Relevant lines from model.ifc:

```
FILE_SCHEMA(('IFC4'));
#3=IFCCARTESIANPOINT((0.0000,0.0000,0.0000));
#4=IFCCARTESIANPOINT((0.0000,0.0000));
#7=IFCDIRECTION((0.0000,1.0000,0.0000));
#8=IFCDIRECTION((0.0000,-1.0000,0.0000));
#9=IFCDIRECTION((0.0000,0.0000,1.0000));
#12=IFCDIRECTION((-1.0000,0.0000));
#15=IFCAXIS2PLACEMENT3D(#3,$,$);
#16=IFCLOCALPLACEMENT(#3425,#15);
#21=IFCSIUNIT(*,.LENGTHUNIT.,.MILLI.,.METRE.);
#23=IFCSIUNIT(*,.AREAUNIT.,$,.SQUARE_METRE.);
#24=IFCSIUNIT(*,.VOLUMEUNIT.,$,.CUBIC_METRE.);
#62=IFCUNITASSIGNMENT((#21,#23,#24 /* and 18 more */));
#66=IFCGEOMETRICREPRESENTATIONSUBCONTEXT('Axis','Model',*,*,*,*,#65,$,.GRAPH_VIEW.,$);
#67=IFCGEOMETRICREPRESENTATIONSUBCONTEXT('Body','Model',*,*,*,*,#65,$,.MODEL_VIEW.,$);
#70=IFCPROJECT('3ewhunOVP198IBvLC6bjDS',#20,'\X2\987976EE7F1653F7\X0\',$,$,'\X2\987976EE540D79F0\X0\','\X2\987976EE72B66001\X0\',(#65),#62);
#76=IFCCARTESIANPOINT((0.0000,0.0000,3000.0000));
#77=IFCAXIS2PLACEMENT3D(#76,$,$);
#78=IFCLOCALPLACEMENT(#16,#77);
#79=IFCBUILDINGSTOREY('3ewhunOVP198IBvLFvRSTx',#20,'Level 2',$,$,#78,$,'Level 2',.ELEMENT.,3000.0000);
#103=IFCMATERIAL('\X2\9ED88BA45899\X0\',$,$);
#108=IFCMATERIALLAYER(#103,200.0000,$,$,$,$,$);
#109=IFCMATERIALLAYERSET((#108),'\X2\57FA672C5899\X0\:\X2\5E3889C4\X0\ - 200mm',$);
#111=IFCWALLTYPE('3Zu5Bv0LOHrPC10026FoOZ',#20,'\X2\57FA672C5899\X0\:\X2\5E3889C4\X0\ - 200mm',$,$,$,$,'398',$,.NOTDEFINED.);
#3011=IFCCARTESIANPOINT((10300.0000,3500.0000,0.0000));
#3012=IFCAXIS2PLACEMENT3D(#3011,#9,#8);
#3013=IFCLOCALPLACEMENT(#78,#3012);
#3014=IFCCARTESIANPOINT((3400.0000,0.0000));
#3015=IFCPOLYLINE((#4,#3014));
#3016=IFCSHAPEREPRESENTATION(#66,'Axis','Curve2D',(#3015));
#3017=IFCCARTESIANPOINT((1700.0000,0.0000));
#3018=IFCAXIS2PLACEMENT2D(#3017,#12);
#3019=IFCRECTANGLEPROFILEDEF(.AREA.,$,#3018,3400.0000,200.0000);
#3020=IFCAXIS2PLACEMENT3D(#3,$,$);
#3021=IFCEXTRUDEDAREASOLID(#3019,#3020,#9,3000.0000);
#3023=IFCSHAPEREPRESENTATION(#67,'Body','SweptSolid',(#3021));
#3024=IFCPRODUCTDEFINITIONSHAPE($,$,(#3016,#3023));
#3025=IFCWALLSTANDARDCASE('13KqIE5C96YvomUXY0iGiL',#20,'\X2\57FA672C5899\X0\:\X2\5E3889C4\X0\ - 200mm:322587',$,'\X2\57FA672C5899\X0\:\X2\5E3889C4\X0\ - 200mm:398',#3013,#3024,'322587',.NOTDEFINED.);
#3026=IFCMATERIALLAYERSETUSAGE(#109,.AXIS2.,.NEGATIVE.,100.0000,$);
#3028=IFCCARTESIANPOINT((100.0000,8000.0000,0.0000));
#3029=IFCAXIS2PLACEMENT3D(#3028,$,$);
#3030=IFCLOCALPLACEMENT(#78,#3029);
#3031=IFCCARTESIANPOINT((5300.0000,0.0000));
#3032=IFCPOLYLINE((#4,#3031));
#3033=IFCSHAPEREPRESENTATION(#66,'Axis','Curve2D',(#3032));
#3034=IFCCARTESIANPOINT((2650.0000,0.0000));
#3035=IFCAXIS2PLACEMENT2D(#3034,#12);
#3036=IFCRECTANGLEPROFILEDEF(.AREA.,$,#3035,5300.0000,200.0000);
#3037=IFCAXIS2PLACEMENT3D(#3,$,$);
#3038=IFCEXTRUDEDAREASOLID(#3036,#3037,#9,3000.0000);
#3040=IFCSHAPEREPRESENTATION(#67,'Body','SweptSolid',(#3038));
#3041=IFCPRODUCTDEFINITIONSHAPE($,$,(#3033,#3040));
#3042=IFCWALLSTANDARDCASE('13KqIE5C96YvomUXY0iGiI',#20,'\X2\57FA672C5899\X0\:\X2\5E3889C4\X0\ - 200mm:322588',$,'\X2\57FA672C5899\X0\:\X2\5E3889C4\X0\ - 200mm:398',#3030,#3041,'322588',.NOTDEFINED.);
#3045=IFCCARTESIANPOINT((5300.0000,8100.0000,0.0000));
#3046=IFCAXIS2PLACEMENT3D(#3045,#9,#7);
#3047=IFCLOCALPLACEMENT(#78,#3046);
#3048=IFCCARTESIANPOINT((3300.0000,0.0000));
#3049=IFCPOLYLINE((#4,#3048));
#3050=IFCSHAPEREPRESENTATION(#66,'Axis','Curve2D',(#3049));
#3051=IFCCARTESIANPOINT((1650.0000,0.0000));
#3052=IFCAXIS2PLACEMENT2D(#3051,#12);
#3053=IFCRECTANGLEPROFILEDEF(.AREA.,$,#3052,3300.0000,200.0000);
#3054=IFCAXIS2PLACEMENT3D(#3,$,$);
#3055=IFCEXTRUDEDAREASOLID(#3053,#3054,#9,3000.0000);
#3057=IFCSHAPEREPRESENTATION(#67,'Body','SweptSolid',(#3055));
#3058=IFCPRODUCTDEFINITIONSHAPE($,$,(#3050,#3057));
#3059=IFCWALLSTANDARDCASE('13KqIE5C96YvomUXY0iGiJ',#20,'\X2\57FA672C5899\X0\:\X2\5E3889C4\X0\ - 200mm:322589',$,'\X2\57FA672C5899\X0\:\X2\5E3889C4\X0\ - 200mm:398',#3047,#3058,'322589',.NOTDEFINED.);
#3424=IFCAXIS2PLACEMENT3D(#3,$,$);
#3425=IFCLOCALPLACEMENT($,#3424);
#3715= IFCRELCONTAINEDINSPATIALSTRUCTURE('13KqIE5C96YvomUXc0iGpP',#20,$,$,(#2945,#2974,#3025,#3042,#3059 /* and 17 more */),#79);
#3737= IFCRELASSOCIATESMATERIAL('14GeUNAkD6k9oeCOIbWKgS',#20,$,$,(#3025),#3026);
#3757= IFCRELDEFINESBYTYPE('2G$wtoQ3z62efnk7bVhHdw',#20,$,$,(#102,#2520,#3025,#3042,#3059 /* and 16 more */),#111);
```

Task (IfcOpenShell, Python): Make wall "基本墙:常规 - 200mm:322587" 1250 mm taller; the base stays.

```python
import ifcopenshell
import ifcopenshell.geom
import ifcopenshell.util.representation
import ifcopenshell.util.shape
import ifcopenshell.util.unit

model = ifcopenshell.open("model.ifc")
unit_scale = ifcopenshell.util.unit.calculate_unit_scale(model)
settings = ifcopenshell.geom.settings()


def volume(element):
    """Net volume in cubic metres, openings subtracted."""
    shape = ifcopenshell.geom.create_shape(settings, element)
    return ifcopenshell.util.shape.get_volume(shape.geometry)


wall = model.by_guid("13KqIE5C96YvomUXY0iGiL")
before = volume(wall)

body = ifcopenshell.util.representation.get_representation(wall, "Model", "Body")
solid = body.Items[0]
old_height = solid.Depth
solid.Depth += 1.25 / unit_scale
after = volume(wall)

print(f"height {old_height:g} -> {solid.Depth:g}, volume {before:.3f} -> {after:.3f} m3")

model.write("model_rev.ifc")
```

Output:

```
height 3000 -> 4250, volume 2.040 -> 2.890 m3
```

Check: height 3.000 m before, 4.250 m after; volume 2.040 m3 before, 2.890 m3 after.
